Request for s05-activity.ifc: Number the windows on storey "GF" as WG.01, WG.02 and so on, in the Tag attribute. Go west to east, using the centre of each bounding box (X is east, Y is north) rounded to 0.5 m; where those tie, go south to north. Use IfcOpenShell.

First a look at what the model holds.

```python
import ifcopenshell
import ifcopenshell.util.element
import ifcopenshell.util.placement

model = ifcopenshell.open("s05-activity.ifc")
print(model.schema)
storey = next(s for s in model.by_type("IfcBuildingStorey") if s.Name == "GF")
windows = [e for e in ifcopenshell.util.element.get_decomposition(storey) if e.is_a("IfcWindow")]
for e in sorted(windows, key=lambda e: e.id()):
    origin = ifcopenshell.util.placement.get_local_placement(e.ObjectPlacement)[:3, 3]
    print(e.id(), e.Tag, e.Name, origin.round(2) + 0.0, sep=" | ")
```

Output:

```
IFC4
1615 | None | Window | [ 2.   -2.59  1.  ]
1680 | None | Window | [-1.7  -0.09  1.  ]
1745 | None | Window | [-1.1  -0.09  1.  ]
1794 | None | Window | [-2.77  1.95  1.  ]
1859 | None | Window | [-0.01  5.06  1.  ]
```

```python
import ifcopenshell
import ifcopenshell.geom
import ifcopenshell.util.element
import ifcopenshell.util.shape

model = ifcopenshell.open("s05-activity.ifc")
settings = ifcopenshell.geom.settings()
settings.set("use-world-coords", True)


def centre(element):
    shape = ifcopenshell.geom.create_shape(settings, element)
    return ifcopenshell.util.shape.get_bbox_centroid(shape.geometry)


storey = next(s for s in model.by_type("IfcBuildingStorey") if s.Name == "GF")
windows = [e for e in ifcopenshell.util.element.get_decomposition(storey) if e.is_a("IfcWindow")]

# Insertion points can sit at a corner or the storey origin, so sort by the geometry (in metres).
centres = {e: centre(e) for e in windows}
windows.sort(key=lambda e: (round(centres[e][0] / 0.5), centres[e][1]))

for i, e in enumerate(windows, start=1):
    number = f"WG.{i:02d}"
    e.Tag = number
    print(e.id(), number)

model.write("s05-activity_rev.ifc")
```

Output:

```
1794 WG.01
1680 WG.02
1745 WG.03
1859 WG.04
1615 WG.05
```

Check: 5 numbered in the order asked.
